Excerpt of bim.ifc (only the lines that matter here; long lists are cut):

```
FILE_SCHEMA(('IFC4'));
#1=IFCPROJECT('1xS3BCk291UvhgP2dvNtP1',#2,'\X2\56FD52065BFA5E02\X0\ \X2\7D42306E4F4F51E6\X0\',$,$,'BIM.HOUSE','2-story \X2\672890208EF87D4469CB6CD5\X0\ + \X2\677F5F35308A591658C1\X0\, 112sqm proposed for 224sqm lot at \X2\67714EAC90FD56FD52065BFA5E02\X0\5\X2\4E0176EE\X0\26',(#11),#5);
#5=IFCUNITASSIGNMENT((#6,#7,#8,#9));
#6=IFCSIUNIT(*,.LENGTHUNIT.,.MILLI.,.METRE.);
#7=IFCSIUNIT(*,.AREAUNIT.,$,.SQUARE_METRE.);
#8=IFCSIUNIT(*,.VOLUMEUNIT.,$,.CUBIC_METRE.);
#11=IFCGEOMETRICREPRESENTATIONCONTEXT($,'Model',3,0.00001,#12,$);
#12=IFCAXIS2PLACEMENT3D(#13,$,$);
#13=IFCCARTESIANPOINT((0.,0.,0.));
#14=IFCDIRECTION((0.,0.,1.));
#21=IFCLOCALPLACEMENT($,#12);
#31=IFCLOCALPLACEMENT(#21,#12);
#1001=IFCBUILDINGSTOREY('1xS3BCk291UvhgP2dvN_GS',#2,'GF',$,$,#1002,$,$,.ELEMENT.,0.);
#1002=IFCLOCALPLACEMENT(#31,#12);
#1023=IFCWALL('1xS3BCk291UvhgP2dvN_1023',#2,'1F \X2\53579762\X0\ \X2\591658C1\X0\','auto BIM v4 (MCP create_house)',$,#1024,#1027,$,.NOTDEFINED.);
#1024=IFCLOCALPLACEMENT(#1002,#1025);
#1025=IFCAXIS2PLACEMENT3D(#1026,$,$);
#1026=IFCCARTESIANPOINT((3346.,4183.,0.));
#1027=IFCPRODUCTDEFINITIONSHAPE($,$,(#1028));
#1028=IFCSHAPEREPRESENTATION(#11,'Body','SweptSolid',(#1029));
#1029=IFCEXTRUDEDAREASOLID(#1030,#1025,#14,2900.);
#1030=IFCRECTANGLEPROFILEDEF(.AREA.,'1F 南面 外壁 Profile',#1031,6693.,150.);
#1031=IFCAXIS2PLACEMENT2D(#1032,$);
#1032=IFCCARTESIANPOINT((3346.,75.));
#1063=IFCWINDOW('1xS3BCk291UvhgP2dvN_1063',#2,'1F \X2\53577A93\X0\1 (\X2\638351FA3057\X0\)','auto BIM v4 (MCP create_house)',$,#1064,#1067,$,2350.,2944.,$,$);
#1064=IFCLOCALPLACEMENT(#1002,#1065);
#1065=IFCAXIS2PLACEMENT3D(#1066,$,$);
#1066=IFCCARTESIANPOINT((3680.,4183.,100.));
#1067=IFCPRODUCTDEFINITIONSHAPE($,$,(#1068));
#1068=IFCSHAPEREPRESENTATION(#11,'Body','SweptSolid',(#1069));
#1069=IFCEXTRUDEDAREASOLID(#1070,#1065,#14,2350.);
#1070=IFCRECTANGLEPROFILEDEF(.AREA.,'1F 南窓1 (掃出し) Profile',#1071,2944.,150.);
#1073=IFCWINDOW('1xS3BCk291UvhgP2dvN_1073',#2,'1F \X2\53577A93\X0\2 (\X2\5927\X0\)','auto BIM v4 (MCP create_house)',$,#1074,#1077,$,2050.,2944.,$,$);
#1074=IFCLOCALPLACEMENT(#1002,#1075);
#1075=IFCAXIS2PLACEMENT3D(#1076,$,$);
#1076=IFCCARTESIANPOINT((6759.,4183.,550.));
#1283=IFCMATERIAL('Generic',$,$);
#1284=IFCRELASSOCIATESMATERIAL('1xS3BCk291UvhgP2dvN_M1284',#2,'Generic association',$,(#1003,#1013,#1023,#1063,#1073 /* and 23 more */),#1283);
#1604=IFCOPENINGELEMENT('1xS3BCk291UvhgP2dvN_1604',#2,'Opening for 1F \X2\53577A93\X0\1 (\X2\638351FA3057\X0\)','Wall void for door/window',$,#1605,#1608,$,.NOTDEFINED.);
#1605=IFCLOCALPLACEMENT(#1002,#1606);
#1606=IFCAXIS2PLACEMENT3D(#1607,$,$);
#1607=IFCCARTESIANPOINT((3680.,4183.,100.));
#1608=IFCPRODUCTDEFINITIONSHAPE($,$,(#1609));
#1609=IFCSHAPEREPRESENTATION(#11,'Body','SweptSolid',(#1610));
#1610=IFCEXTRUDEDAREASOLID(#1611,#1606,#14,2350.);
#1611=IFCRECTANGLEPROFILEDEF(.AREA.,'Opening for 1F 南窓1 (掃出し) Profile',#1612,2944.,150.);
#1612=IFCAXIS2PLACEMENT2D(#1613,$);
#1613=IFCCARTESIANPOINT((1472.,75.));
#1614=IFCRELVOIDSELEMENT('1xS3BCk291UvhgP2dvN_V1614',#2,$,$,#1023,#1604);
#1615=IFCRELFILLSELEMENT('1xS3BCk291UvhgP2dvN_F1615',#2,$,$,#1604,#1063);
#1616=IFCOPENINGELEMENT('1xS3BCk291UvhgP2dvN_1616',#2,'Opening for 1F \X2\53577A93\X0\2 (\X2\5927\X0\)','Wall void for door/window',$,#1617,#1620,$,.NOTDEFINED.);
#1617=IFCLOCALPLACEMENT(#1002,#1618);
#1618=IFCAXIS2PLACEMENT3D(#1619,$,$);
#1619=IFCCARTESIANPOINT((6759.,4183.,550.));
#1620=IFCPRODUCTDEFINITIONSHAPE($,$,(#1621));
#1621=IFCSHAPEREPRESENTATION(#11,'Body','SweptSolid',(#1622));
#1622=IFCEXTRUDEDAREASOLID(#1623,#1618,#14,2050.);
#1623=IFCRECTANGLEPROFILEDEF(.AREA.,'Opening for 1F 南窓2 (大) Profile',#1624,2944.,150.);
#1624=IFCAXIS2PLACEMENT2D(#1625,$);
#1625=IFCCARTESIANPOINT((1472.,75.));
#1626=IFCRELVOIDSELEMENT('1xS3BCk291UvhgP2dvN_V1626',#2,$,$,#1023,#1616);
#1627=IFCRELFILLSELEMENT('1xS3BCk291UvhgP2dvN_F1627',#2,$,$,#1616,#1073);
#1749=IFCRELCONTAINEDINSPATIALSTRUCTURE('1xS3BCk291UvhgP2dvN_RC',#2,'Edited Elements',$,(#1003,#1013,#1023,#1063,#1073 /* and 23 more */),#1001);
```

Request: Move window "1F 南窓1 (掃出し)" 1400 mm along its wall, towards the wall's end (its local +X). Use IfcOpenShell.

```python
import ifcopenshell
import ifcopenshell.api.geometry
import ifcopenshell.util.placement
import ifcopenshell.util.unit

model = ifcopenshell.open("bim.ifc")
unit_scale = ifcopenshell.util.unit.calculate_unit_scale(model)

window = model.by_id(1063)
opening = window.FillsVoids[0].RelatingOpeningElement
wall = opening.VoidsElements[0].RelatingBuildingElement

wall_matrix = ifcopenshell.util.placement.get_local_placement(wall.ObjectPlacement)
shift = wall_matrix[:3, 0] * 1.4 / unit_scale
before = ifcopenshell.util.placement.get_local_placement(window.ObjectPlacement)[:3, 3].copy()

# The window is not placed relative to its opening, so move both.
for product in (opening, window):
    matrix = ifcopenshell.util.placement.get_local_placement(product.ObjectPlacement)
    matrix[:3, 3] += shift
    ifcopenshell.api.geometry.edit_object_placement(model, product=product, matrix=matrix, is_si=False)

after = ifcopenshell.util.placement.get_local_placement(window.ObjectPlacement)[:3, 3]
print("window moved by", (after - before).round(3) + 0.0)

model.write("bim_v2.ifc")
```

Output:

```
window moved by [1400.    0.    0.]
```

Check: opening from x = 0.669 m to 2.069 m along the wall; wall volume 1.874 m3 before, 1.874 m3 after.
